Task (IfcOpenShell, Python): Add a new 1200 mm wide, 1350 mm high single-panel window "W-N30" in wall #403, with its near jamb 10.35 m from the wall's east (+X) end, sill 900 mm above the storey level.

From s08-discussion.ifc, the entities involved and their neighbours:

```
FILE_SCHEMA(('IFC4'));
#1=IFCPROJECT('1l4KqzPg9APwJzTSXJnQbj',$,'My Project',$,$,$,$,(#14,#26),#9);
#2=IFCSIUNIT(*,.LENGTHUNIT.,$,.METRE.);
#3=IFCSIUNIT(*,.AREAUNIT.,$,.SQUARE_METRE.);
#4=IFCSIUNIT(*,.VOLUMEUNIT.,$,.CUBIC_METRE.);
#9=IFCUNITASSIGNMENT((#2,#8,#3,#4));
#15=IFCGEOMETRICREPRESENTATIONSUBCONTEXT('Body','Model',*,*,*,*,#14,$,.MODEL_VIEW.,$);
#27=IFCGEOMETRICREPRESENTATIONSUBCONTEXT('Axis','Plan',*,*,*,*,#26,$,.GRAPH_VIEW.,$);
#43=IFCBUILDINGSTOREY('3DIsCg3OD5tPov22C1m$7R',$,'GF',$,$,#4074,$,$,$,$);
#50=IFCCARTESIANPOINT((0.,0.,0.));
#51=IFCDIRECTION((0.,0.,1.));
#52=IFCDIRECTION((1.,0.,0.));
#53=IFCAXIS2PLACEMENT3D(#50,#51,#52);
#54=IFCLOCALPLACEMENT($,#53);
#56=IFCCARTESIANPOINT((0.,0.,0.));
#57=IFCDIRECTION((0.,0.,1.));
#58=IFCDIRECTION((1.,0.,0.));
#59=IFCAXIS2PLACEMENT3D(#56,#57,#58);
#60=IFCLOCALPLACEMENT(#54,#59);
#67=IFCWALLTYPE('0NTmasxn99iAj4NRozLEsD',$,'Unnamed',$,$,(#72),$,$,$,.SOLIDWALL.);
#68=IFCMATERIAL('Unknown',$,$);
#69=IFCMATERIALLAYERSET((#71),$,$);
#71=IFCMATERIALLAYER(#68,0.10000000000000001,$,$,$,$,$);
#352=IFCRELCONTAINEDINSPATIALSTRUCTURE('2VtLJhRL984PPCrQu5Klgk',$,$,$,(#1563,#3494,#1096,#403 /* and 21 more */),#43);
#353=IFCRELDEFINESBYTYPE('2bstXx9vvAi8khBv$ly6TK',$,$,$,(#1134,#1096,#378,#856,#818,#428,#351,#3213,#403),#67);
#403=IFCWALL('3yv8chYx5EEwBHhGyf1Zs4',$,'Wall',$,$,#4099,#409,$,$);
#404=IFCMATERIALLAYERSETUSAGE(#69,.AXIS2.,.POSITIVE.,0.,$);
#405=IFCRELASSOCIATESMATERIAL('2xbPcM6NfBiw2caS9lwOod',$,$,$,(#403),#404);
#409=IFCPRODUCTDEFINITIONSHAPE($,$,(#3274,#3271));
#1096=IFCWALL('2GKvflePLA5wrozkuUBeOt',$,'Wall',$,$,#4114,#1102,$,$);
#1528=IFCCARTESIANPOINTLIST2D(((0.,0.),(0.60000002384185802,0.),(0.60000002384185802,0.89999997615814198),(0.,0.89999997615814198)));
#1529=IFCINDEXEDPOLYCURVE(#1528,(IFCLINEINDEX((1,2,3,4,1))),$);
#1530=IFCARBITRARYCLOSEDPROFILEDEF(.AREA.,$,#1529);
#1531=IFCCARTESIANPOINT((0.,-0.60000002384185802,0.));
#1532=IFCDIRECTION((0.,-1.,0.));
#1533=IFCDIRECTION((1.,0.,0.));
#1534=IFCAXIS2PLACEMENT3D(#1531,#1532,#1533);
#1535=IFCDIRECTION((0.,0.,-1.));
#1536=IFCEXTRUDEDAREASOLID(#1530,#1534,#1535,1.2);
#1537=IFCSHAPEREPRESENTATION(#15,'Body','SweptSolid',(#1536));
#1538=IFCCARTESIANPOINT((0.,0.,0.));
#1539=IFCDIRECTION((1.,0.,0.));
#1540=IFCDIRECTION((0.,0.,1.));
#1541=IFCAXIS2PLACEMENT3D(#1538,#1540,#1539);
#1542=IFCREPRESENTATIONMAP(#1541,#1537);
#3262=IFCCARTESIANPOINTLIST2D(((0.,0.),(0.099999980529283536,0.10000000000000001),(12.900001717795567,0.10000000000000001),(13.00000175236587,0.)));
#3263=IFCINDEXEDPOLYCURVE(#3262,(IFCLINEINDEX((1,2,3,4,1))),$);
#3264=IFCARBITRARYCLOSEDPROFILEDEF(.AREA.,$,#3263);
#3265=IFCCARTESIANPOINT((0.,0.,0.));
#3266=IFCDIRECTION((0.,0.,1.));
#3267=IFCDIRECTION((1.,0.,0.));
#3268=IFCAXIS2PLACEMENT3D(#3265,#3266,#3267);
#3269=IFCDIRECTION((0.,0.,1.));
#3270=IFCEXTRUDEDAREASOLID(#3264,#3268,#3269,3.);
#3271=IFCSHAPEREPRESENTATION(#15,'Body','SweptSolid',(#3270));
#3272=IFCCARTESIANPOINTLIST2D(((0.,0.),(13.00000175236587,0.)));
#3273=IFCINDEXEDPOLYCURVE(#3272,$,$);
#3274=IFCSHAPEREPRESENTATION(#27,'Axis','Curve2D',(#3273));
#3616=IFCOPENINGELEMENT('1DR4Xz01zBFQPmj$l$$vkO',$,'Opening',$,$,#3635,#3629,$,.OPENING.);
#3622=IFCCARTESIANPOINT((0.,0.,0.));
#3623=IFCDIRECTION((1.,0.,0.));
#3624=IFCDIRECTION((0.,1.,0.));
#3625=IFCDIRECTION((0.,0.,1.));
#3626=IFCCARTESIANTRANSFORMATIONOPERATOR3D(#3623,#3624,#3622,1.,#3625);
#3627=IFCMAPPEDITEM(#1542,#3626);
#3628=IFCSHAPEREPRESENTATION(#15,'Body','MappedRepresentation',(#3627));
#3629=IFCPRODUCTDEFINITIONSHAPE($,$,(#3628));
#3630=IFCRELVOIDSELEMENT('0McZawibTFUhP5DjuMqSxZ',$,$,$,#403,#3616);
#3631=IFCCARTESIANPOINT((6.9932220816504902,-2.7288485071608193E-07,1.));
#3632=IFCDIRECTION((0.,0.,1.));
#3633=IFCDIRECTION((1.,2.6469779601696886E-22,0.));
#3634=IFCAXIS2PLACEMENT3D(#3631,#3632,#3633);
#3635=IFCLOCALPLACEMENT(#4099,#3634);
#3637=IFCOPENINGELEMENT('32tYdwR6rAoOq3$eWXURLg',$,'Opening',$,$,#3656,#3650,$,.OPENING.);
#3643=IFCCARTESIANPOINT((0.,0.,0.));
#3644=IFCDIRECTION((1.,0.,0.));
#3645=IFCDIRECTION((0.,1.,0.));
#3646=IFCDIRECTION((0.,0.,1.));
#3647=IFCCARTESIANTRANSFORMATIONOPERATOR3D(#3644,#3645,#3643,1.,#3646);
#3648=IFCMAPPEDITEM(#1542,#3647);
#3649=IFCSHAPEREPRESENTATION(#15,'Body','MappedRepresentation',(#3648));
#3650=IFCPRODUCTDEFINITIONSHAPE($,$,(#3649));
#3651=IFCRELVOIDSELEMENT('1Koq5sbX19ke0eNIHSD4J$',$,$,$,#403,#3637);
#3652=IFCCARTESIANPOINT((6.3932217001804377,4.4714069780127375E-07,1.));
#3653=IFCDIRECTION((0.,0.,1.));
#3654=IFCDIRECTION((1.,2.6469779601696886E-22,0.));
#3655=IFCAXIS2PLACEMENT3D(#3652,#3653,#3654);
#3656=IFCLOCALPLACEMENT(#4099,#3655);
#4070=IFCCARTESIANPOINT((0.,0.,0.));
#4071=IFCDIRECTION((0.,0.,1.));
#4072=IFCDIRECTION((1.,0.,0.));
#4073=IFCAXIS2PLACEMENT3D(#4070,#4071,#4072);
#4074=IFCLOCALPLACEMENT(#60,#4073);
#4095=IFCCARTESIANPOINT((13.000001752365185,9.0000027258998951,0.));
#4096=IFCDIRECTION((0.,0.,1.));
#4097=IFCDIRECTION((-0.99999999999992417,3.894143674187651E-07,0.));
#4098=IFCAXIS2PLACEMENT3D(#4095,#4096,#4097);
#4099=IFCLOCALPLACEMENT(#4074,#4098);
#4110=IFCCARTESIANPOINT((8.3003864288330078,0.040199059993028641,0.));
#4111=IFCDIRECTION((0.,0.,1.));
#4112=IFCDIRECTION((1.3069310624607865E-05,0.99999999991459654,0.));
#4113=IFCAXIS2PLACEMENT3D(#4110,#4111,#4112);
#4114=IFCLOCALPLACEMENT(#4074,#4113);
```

```python
import numpy as np
import ifcopenshell
import ifcopenshell.api.feature
import ifcopenshell.api.geometry
import ifcopenshell.api.root
import ifcopenshell.api.spatial
import ifcopenshell.geom
import ifcopenshell.util.element
import ifcopenshell.util.placement
import ifcopenshell.util.representation
import ifcopenshell.util.shape
import ifcopenshell.util.unit

model = ifcopenshell.open("s08-discussion.ifc")
unit_scale = ifcopenshell.util.unit.calculate_unit_scale(model)
settings = ifcopenshell.geom.settings()


def volume(element):
    """Net volume in cubic metres, openings subtracted."""
    shape = ifcopenshell.geom.create_shape(settings, element)
    return ifcopenshell.util.shape.get_volume(shape.geometry)


wall = model.by_guid("3yv8chYx5EEwBHhGyf1Zs4")
storey = ifcopenshell.util.element.get_container(wall, ifc_class="IfcBuildingStorey")
context = ifcopenshell.util.representation.get_context(model, "Model", "Body", "MODEL_VIEW")
before = volume(wall)

width, height, from_end, sill = 1.2, 1.35, 10.35, 0.9  # metres

# The wall runs along its own X axis, and the end named is its -X end.
wall_shape = ifcopenshell.geom.create_shape(settings, wall)
x, y, z = ifcopenshell.util.shape.get_vertices(wall_shape.geometry).T
start = x.min() + from_end
face, thickness = float(y.min()), float(y.max() - y.min())
wall_matrix = ifcopenshell.util.placement.get_local_placement(wall.ObjectPlacement)
level = ifcopenshell.util.placement.get_local_placement(storey.ObjectPlacement)[2, 3]


def in_wall(x, y):
    """Placement at x, y metres in the wall's axes, at sill height."""
    matrix = wall_matrix.copy()
    matrix[:, 3] = wall_matrix @ np.array([x / unit_scale, y / unit_scale, 0.0, 1.0])
    matrix[2, 3] = level + sill / unit_scale
    return matrix


# Opening: a box that overshoots both wall faces by 50 mm.
opening = ifcopenshell.api.root.create_entity(model, ifc_class="IfcOpeningElement", predefined_type="OPENING")
box = ifcopenshell.api.geometry.add_wall_representation(
    model, context=context, length=width, height=height, thickness=thickness + 0.1
)
ifcopenshell.api.geometry.assign_representation(model, product=opening, representation=box)
ifcopenshell.api.geometry.edit_object_placement(model, product=opening, matrix=in_wall(start, face - 0.05), is_si=False)
ifcopenshell.api.feature.add_feature(model, feature=opening, element=wall)

window = ifcopenshell.api.root.create_entity(model, ifc_class="IfcWindow", name="W-N30", predefined_type="WINDOW")
window.OverallWidth, window.OverallHeight = width / unit_scale, height / unit_scale
window.PartitioningType = "SINGLE_PANEL"
body = ifcopenshell.api.geometry.add_window_representation(
    model,
    context=context,
    overall_width=window.OverallWidth,
    overall_height=window.OverallHeight,
    partition_type="SINGLE_PANEL",
)
ifcopenshell.api.geometry.assign_representation(model, product=window, representation=body)
ifcopenshell.api.spatial.assign_container(model, products=[window], relating_structure=storey)
ifcopenshell.api.feature.add_filling(model, opening=opening, element=window)

# Centre the window in the wall's thickness.
ifcopenshell.api.geometry.edit_object_placement(model, product=window, matrix=in_wall(start, face), is_si=False)
window_shape = ifcopenshell.geom.create_shape(settings, window)
depth = ifcopenshell.util.shape.get_vertices(window_shape.geometry)[:, 1]
offset = face + thickness / 2 - (depth.min() + depth.max()) / 2
ifcopenshell.api.geometry.edit_object_placement(model, product=window, matrix=in_wall(start, offset), is_si=False)

after = volume(wall)

print(f"wall volume {before:.3f} -> {after:.3f} m3")

model.write("s08-discussion-out.ifc")
```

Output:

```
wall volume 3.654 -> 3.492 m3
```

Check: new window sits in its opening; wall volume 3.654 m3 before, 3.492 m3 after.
